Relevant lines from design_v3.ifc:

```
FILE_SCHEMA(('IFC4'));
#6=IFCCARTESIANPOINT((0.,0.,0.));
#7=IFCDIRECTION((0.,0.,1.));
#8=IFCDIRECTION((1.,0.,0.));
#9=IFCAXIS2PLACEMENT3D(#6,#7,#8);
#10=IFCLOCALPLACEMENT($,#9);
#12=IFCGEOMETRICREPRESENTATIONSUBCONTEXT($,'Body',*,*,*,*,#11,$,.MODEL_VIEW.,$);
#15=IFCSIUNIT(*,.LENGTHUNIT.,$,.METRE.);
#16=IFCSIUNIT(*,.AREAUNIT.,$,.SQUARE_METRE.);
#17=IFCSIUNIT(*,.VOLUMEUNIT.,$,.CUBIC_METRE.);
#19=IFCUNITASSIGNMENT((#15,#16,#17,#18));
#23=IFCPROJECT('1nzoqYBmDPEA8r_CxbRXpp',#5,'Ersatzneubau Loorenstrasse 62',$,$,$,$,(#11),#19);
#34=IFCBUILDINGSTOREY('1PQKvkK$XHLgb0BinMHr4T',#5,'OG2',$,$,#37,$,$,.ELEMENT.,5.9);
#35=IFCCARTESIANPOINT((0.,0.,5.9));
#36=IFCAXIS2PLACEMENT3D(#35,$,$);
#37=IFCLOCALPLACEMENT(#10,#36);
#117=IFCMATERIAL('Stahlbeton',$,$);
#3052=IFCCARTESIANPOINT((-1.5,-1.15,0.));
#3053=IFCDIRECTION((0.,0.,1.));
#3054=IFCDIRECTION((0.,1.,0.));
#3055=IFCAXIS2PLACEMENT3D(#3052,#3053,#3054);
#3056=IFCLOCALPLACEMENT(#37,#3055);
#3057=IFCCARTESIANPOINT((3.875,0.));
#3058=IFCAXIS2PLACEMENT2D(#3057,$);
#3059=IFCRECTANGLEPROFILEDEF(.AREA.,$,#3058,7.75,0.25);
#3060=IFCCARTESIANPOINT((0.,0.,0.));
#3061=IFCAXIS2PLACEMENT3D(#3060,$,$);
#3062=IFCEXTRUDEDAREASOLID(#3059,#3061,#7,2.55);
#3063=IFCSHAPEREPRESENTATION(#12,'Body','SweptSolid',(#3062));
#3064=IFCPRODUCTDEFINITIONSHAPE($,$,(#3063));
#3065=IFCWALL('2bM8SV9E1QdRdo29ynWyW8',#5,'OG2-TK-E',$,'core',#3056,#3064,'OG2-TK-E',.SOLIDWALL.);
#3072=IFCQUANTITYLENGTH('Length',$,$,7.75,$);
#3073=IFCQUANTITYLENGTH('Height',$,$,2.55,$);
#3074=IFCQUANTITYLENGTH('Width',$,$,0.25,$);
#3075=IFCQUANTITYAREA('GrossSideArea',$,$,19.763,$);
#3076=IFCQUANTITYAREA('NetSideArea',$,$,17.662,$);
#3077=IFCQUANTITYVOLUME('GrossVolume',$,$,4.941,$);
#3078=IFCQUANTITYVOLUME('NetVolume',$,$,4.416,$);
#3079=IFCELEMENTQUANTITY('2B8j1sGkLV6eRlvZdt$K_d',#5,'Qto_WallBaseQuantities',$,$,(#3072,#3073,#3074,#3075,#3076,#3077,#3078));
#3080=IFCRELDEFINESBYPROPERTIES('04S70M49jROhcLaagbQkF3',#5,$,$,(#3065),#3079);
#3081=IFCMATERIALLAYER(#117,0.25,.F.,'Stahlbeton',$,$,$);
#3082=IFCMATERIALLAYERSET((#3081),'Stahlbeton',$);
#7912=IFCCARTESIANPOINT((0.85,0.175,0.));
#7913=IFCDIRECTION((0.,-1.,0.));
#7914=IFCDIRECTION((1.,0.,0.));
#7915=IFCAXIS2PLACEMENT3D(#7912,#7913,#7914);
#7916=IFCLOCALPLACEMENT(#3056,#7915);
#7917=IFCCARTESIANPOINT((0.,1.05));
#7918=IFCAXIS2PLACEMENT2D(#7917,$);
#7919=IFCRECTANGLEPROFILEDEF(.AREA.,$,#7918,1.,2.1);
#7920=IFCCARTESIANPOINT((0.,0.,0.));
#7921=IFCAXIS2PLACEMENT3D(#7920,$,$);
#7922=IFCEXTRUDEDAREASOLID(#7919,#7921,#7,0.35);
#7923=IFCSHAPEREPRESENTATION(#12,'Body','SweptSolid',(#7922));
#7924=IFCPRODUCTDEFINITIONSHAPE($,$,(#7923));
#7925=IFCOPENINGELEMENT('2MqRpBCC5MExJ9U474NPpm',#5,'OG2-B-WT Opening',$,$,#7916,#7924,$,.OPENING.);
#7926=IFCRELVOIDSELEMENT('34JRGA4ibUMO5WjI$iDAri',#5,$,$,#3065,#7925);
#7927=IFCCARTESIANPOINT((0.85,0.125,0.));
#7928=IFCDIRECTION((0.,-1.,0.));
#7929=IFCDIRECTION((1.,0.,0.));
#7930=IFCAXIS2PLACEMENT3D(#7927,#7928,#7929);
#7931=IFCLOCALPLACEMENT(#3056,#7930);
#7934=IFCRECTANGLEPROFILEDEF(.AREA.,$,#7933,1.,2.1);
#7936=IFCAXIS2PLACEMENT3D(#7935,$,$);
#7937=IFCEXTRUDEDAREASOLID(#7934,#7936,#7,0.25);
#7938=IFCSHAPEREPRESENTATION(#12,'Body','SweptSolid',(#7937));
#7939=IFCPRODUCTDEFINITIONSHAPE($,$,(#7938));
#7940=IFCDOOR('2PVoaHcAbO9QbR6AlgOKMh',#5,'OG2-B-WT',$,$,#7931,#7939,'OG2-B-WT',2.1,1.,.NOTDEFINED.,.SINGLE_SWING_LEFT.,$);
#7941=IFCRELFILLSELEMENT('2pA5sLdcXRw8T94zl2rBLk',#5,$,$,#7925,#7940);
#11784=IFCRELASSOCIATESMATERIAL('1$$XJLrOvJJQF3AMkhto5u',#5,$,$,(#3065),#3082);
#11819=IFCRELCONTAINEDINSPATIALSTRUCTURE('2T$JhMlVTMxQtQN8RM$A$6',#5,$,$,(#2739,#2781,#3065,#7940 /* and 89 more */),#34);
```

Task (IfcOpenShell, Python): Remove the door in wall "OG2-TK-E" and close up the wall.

```python
import ifcopenshell
import ifcopenshell.api.feature
import ifcopenshell.api.pset
import ifcopenshell.api.root
import ifcopenshell.geom
import ifcopenshell.util.element
import ifcopenshell.util.shape
import ifcopenshell.util.unit

model = ifcopenshell.open("design_v3.ifc")
area_scale = ifcopenshell.util.unit.calculate_unit_scale(model, "AREAUNIT")
volume_scale = ifcopenshell.util.unit.calculate_unit_scale(model, "VOLUMEUNIT")
settings = ifcopenshell.geom.settings()


def volume(element):
    """Net volume in cubic metres, openings subtracted."""
    shape = ifcopenshell.geom.create_shape(settings, element)
    return ifcopenshell.util.shape.get_volume(shape.geometry)


door = model.by_guid("2PVoaHcAbO9QbR6AlgOKMh")
opening = door.FillsVoids[0].RelatingOpeningElement
wall = opening.VoidsElements[0].RelatingBuildingElement
before = volume(wall)

ifcopenshell.api.root.remove_product(model, product=door)
ifcopenshell.api.feature.remove_feature(model, feature=opening)

after = volume(wall)
thickness = 0.25  # wall thickness in metres

# Update the wall's stored quantities.
qto = model.by_id(ifcopenshell.util.element.get_pset(wall, "Qto_WallBaseQuantities", should_inherit=False)["id"])
ifcopenshell.api.pset.edit_qto(model, qto=qto, properties={
    "NetSideArea": after / thickness / area_scale,
    "NetVolume": after / volume_scale,
})

print(f"wall volume {before:.3f} -> {after:.3f} m3")

model.write("design_v3_updated.ifc")
```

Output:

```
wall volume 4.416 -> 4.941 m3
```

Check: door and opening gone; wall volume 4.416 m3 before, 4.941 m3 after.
